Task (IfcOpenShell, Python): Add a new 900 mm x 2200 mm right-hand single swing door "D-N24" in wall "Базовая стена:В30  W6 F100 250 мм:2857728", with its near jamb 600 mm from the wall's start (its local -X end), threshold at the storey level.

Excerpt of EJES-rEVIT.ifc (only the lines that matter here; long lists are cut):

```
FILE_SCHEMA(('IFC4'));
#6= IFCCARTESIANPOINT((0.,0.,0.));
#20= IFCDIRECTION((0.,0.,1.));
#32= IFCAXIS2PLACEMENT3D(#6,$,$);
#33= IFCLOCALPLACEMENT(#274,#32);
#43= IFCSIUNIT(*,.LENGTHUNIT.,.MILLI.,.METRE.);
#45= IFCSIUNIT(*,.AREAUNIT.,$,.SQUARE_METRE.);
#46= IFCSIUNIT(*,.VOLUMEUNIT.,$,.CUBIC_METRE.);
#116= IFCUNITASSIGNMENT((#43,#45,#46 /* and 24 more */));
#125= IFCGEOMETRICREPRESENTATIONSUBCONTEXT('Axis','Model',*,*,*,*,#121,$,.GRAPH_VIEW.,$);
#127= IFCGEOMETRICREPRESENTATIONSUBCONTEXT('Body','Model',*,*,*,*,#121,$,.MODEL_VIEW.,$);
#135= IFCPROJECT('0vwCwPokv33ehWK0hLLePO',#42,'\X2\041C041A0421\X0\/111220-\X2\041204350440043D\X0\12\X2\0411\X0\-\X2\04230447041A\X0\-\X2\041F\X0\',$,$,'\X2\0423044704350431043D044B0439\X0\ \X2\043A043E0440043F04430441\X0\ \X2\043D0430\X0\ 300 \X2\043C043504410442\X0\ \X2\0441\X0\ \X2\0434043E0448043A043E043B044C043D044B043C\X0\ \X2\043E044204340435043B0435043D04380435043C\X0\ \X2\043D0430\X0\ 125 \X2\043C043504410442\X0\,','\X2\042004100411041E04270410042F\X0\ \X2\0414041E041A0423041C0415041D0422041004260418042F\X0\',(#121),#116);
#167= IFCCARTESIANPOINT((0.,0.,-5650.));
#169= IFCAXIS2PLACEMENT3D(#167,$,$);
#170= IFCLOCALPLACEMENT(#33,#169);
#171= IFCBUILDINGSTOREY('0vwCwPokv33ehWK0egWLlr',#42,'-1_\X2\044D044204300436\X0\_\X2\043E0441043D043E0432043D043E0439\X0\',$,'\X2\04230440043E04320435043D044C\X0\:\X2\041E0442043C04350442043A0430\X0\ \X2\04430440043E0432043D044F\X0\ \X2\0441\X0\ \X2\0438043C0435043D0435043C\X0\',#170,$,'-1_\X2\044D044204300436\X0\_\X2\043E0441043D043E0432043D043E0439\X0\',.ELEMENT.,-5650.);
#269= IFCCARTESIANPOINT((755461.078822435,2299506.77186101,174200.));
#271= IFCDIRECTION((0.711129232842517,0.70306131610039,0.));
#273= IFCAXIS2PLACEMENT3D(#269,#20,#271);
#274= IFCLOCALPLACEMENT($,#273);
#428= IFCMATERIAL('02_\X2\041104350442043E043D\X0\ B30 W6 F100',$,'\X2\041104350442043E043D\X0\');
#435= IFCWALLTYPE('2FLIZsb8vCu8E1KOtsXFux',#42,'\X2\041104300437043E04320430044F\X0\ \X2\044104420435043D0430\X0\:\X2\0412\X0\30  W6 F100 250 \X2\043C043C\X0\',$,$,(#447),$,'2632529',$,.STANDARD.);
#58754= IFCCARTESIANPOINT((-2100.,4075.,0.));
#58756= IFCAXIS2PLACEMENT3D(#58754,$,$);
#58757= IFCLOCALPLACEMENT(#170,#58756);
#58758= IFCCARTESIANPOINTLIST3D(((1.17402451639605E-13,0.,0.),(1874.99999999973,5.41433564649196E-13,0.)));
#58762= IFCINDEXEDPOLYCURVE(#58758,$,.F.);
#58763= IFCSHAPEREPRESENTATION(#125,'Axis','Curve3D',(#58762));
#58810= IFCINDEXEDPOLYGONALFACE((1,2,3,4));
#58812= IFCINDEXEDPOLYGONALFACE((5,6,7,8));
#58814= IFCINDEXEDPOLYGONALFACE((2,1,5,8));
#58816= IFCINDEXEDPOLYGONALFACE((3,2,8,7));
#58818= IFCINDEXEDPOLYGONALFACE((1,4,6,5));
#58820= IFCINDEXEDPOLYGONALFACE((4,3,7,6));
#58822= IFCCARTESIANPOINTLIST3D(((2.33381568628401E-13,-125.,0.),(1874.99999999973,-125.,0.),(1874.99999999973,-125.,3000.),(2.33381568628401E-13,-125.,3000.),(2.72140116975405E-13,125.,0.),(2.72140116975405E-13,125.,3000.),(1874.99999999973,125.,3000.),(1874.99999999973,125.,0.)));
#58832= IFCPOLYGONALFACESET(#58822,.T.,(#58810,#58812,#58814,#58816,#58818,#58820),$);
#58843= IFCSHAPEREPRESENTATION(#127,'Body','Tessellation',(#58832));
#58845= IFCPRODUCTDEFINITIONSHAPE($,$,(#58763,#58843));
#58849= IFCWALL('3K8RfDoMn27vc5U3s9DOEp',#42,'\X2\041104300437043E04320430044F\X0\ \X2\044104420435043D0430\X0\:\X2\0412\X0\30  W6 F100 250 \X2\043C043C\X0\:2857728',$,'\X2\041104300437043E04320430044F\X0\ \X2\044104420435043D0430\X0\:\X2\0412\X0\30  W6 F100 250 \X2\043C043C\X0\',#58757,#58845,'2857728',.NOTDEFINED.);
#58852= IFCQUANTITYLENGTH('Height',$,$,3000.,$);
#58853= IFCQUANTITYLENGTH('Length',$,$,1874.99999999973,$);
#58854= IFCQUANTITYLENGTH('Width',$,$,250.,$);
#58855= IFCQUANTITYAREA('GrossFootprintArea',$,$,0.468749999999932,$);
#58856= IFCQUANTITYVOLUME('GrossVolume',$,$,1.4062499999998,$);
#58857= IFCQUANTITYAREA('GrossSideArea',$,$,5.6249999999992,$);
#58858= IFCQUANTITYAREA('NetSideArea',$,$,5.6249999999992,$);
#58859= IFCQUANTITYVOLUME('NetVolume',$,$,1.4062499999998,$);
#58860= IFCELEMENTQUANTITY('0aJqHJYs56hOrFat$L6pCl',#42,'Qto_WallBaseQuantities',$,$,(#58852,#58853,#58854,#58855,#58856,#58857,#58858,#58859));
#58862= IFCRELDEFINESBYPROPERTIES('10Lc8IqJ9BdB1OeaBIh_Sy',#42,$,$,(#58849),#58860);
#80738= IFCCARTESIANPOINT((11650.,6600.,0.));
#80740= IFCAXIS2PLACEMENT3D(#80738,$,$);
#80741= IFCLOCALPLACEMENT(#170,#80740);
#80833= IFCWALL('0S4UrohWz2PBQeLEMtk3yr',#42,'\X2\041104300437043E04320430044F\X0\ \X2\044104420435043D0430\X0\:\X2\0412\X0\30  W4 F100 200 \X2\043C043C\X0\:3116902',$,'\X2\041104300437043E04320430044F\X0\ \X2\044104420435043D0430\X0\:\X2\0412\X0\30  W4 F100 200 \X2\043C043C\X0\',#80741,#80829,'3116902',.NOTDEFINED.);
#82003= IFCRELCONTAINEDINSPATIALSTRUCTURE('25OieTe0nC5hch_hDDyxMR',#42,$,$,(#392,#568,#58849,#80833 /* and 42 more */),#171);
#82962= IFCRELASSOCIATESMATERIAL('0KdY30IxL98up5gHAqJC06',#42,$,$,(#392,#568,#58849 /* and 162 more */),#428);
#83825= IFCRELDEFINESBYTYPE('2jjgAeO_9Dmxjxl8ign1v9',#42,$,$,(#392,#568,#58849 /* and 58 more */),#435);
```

```python
import numpy as np
import ifcopenshell
import ifcopenshell.api.feature
import ifcopenshell.api.geometry
import ifcopenshell.api.pset
import ifcopenshell.api.root
import ifcopenshell.api.spatial
import ifcopenshell.geom
import ifcopenshell.util.element
import ifcopenshell.util.placement
import ifcopenshell.util.representation
import ifcopenshell.util.shape
import ifcopenshell.util.unit

model = ifcopenshell.open("EJES-rEVIT.ifc")
unit_scale = ifcopenshell.util.unit.calculate_unit_scale(model)
area_scale = ifcopenshell.util.unit.calculate_unit_scale(model, "AREAUNIT")
volume_scale = ifcopenshell.util.unit.calculate_unit_scale(model, "VOLUMEUNIT")
settings = ifcopenshell.geom.settings()


def volume(element):
    """Net volume in cubic metres, openings subtracted."""
    shape = ifcopenshell.geom.create_shape(settings, element)
    return ifcopenshell.util.shape.get_volume(shape.geometry)


wall = model.by_guid("3K8RfDoMn27vc5U3s9DOEp")
storey = ifcopenshell.util.element.get_container(wall, ifc_class="IfcBuildingStorey")
context = ifcopenshell.util.representation.get_context(model, "Model", "Body", "MODEL_VIEW")
before = volume(wall)

width, height, from_end, sill = 0.9, 2.2, 0.6, 0.0  # metres

# The wall runs along its own X axis, and the end named is its -X end.
wall_shape = ifcopenshell.geom.create_shape(settings, wall)
x, y, z = ifcopenshell.util.shape.get_vertices(wall_shape.geometry).T
start = x.min() + from_end
face, thickness = float(y.min()), float(y.max() - y.min())
wall_matrix = ifcopenshell.util.placement.get_local_placement(wall.ObjectPlacement)
level = ifcopenshell.util.placement.get_local_placement(storey.ObjectPlacement)[2, 3]


def in_wall(x, y):
    """Placement at x, y metres in the wall's axes, at sill height."""
    matrix = wall_matrix.copy()
    matrix[:, 3] = wall_matrix @ np.array([x / unit_scale, y / unit_scale, 0.0, 1.0])
    matrix[2, 3] = level + sill / unit_scale
    return matrix


# Opening: a box that overshoots both wall faces by 50 mm.
opening = ifcopenshell.api.root.create_entity(model, ifc_class="IfcOpeningElement", predefined_type="OPENING")
box = ifcopenshell.api.geometry.add_wall_representation(
    model, context=context, length=width, height=height, thickness=thickness + 0.1
)
ifcopenshell.api.geometry.assign_representation(model, product=opening, representation=box)
ifcopenshell.api.geometry.edit_object_placement(model, product=opening, matrix=in_wall(start, face - 0.05), is_si=False)
ifcopenshell.api.feature.add_feature(model, feature=opening, element=wall)

door = ifcopenshell.api.root.create_entity(model, ifc_class="IfcDoor", name="D-N24", predefined_type="DOOR")
door.OverallWidth, door.OverallHeight = width / unit_scale, height / unit_scale
door.OperationType = "SINGLE_SWING_RIGHT"
body = ifcopenshell.api.geometry.add_door_representation(
    model,
    context=context,
    overall_width=door.OverallWidth,
    overall_height=door.OverallHeight,
    operation_type="SINGLE_SWING_RIGHT",
    lining_properties={"LiningDepth": thickness / unit_scale, "ThresholdDepth": thickness / unit_scale},
)
ifcopenshell.api.geometry.assign_representation(model, product=door, representation=body)
ifcopenshell.api.spatial.assign_container(model, products=[door], relating_structure=storey)
ifcopenshell.api.feature.add_filling(model, opening=opening, element=door)

# The lining spans the wall, so the door starts at the wall face.
ifcopenshell.api.geometry.edit_object_placement(model, product=door, matrix=in_wall(start, face), is_si=False)

after = volume(wall)

# Update the wall's stored quantities.
qto = model.by_id(ifcopenshell.util.element.get_pset(wall, "Qto_WallBaseQuantities", should_inherit=False)["id"])
ifcopenshell.api.pset.edit_qto(model, qto=qto, properties={
    "NetSideArea": after / thickness / area_scale,
    "NetVolume": after / volume_scale,
})

print(f"wall volume {before:.3f} -> {after:.3f} m3")

model.write("EJES-rEVIT_edited.ifc")
```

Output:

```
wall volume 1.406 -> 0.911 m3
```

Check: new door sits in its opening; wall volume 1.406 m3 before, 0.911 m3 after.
